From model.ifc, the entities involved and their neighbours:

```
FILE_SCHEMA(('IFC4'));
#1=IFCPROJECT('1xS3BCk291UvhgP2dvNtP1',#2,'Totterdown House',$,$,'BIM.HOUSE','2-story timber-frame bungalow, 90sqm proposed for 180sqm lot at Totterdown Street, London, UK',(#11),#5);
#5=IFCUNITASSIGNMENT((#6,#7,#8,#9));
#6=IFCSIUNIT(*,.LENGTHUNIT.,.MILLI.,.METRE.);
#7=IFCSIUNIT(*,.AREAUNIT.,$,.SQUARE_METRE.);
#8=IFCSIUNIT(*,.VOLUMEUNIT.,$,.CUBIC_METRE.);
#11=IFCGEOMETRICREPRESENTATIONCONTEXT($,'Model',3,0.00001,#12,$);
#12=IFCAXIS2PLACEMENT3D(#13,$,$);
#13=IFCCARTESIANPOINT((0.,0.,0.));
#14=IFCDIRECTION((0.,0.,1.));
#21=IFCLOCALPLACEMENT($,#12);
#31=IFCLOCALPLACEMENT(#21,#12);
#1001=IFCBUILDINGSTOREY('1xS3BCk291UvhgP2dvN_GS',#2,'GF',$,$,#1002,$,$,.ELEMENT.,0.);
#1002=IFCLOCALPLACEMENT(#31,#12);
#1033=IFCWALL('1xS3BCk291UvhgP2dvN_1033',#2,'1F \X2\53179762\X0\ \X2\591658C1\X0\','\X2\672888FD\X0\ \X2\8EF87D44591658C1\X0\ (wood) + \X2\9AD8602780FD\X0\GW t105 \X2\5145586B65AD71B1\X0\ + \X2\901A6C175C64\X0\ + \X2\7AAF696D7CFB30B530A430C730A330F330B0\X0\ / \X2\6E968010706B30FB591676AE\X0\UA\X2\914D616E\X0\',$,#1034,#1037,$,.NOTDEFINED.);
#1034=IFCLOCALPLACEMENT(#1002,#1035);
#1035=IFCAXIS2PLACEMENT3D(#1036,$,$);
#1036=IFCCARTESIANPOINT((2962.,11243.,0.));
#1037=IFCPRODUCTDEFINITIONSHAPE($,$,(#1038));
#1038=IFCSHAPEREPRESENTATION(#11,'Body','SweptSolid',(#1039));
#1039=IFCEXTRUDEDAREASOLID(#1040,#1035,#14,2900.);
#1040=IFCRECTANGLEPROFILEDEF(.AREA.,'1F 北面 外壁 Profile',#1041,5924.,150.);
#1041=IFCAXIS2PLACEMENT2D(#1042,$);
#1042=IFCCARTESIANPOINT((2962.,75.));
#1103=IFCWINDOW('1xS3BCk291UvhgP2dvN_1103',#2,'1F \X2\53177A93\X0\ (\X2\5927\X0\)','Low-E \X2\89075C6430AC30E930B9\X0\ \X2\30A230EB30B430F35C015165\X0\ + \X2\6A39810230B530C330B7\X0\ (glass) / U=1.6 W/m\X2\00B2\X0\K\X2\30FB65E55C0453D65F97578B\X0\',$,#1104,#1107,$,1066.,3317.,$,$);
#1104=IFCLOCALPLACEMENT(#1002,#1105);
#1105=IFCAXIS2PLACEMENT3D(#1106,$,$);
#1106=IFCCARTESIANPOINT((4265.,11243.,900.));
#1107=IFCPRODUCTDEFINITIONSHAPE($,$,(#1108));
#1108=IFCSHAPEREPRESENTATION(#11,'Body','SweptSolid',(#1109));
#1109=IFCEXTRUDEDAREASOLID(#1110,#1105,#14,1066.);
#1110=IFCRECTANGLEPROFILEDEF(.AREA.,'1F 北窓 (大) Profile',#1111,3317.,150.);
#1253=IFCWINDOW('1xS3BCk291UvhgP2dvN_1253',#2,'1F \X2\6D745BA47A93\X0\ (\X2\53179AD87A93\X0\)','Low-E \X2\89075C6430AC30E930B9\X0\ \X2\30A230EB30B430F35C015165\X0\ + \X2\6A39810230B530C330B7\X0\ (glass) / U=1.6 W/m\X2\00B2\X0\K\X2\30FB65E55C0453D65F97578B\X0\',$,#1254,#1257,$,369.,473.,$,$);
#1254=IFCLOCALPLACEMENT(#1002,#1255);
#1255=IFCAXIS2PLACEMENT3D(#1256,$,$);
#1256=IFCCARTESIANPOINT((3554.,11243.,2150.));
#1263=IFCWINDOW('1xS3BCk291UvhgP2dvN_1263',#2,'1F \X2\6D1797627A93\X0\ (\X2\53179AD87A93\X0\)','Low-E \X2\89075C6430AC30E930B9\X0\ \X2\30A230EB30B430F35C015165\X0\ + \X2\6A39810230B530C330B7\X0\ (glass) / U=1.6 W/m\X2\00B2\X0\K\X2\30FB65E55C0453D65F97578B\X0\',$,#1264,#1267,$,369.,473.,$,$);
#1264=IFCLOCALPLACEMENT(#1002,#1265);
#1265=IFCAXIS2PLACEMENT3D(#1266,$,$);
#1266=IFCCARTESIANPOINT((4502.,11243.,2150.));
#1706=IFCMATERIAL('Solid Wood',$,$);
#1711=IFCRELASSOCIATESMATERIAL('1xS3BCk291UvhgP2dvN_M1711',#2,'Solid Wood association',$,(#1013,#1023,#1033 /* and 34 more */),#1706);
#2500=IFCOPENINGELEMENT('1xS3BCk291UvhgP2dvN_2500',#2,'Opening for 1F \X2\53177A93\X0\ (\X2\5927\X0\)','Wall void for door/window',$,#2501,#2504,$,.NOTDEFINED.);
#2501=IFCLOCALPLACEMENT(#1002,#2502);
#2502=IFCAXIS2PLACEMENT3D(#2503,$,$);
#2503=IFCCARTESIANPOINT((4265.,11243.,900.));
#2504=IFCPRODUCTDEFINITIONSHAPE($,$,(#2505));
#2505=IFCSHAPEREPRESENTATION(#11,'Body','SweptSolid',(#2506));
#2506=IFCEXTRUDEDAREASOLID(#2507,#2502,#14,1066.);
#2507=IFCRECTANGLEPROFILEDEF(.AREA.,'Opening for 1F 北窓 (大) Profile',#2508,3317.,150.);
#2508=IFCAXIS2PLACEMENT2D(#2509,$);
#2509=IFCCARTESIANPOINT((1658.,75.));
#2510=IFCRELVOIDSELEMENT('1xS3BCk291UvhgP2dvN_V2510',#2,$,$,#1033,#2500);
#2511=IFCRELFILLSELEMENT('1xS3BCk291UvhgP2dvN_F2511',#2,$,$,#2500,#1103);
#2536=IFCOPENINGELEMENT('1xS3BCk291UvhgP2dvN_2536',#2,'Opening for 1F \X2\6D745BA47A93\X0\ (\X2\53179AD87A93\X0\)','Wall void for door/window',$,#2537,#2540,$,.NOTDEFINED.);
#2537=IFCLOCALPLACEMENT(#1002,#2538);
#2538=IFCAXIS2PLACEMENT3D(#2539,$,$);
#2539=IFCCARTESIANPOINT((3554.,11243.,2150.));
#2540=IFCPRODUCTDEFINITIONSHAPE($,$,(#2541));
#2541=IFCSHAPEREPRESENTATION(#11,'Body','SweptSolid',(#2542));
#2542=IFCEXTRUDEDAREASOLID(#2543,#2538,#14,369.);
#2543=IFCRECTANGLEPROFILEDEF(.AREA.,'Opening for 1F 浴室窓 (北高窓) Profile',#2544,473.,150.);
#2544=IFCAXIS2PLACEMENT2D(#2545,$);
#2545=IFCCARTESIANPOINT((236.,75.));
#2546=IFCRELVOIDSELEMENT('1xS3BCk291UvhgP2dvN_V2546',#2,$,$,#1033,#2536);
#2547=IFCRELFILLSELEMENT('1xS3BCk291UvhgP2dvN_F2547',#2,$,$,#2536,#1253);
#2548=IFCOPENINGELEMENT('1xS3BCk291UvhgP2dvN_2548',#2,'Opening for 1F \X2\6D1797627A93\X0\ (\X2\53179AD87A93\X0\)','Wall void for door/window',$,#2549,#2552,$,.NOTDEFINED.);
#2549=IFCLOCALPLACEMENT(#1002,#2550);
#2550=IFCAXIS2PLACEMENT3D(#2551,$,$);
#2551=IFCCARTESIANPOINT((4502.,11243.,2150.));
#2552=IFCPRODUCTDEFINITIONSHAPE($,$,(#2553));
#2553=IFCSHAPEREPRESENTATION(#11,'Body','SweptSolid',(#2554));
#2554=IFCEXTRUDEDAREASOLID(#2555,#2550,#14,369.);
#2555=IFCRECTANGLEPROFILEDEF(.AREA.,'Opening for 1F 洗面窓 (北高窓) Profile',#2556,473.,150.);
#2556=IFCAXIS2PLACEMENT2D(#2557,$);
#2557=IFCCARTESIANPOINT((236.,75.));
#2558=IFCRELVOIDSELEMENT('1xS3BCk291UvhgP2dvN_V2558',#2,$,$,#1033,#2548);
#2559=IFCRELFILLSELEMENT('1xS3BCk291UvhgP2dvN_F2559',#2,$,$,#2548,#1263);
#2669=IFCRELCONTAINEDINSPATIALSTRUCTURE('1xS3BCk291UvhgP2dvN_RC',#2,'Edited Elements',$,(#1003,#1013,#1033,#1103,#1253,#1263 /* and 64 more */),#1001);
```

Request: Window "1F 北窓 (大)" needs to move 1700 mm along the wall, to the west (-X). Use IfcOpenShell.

```python
import ifcopenshell
import ifcopenshell.api.geometry
import ifcopenshell.util.placement

model = ifcopenshell.open("model.ifc")

window = model.by_guid("1xS3BCk291UvhgP2dvN_1103")
opening = window.FillsVoids[0].RelatingOpeningElement
wall = opening.VoidsElements[0].RelatingBuildingElement

wall_matrix = ifcopenshell.util.placement.get_local_placement(wall.ObjectPlacement)
shift = wall_matrix[:3, 0] * -1700.0
before = ifcopenshell.util.placement.get_local_placement(window.ObjectPlacement)[:3, 3].copy()

# The window is not placed relative to its opening, so move both.
for product in (opening, window):
    matrix = ifcopenshell.util.placement.get_local_placement(product.ObjectPlacement)
    matrix[:3, 3] += shift
    ifcopenshell.api.geometry.edit_object_placement(model, product=product, matrix=matrix, is_si=False)

after = ifcopenshell.util.placement.get_local_placement(window.ObjectPlacement)[:3, 3]
print("window moved by", (after - before).round(3) + 0.0)

model.write("model_v2.ifc")
```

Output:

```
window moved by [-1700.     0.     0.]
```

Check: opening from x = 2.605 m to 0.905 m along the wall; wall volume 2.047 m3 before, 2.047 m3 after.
